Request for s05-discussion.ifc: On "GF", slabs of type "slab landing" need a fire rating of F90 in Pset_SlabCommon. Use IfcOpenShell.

First a look at what the model holds.

```python
import ifcopenshell
import ifcopenshell.util.element

model = ifcopenshell.open("s05-discussion.ifc")
print(model.schema)
storey = next(s for s in model.by_type("IfcBuildingStorey") if s.Name == "GF")
slabs = [e for e in ifcopenshell.util.element.get_decomposition(storey) if e.is_a("IfcSlab")]
seen = {}
for e in slabs:
    element_type = ifcopenshell.util.element.get_type(e)
    key = (element_type.Name if element_type != e and element_type else None, ifcopenshell.util.element.get_pset(e, "Pset_SlabCommon", "FireRating"))
    seen[key] = seen.get(key, 0) + 1
for (name, value), count in sorted(seen.items(), key=str):
    print(count, "x", name, "|", value)
```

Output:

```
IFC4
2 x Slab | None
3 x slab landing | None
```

```python
import ifcopenshell
import ifcopenshell.api.pset
import ifcopenshell.util.element

model = ifcopenshell.open("s05-discussion.ifc")

storey = next(s for s in model.by_type("IfcBuildingStorey") if s.Name == "GF")
slabs = [e for e in ifcopenshell.util.element.get_decomposition(storey) if e.is_a("IfcSlab")]

count = 0
for e in slabs:
    element_type = ifcopenshell.util.element.get_type(e)
    if element_type in (None, e) or element_type.Name != "slab landing":
        continue
    # add_pset returns the element's existing set when there is one.
    pset = ifcopenshell.api.pset.add_pset(model, product=e, name="Pset_SlabCommon")
    ifcopenshell.api.pset.edit_pset(model, pset=pset, properties={"FireRating": "F90"})
    count += 1

print(count, "slabs updated")

model.write("s05-discussion_edited.ifc")
```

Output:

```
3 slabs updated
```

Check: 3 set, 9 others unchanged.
